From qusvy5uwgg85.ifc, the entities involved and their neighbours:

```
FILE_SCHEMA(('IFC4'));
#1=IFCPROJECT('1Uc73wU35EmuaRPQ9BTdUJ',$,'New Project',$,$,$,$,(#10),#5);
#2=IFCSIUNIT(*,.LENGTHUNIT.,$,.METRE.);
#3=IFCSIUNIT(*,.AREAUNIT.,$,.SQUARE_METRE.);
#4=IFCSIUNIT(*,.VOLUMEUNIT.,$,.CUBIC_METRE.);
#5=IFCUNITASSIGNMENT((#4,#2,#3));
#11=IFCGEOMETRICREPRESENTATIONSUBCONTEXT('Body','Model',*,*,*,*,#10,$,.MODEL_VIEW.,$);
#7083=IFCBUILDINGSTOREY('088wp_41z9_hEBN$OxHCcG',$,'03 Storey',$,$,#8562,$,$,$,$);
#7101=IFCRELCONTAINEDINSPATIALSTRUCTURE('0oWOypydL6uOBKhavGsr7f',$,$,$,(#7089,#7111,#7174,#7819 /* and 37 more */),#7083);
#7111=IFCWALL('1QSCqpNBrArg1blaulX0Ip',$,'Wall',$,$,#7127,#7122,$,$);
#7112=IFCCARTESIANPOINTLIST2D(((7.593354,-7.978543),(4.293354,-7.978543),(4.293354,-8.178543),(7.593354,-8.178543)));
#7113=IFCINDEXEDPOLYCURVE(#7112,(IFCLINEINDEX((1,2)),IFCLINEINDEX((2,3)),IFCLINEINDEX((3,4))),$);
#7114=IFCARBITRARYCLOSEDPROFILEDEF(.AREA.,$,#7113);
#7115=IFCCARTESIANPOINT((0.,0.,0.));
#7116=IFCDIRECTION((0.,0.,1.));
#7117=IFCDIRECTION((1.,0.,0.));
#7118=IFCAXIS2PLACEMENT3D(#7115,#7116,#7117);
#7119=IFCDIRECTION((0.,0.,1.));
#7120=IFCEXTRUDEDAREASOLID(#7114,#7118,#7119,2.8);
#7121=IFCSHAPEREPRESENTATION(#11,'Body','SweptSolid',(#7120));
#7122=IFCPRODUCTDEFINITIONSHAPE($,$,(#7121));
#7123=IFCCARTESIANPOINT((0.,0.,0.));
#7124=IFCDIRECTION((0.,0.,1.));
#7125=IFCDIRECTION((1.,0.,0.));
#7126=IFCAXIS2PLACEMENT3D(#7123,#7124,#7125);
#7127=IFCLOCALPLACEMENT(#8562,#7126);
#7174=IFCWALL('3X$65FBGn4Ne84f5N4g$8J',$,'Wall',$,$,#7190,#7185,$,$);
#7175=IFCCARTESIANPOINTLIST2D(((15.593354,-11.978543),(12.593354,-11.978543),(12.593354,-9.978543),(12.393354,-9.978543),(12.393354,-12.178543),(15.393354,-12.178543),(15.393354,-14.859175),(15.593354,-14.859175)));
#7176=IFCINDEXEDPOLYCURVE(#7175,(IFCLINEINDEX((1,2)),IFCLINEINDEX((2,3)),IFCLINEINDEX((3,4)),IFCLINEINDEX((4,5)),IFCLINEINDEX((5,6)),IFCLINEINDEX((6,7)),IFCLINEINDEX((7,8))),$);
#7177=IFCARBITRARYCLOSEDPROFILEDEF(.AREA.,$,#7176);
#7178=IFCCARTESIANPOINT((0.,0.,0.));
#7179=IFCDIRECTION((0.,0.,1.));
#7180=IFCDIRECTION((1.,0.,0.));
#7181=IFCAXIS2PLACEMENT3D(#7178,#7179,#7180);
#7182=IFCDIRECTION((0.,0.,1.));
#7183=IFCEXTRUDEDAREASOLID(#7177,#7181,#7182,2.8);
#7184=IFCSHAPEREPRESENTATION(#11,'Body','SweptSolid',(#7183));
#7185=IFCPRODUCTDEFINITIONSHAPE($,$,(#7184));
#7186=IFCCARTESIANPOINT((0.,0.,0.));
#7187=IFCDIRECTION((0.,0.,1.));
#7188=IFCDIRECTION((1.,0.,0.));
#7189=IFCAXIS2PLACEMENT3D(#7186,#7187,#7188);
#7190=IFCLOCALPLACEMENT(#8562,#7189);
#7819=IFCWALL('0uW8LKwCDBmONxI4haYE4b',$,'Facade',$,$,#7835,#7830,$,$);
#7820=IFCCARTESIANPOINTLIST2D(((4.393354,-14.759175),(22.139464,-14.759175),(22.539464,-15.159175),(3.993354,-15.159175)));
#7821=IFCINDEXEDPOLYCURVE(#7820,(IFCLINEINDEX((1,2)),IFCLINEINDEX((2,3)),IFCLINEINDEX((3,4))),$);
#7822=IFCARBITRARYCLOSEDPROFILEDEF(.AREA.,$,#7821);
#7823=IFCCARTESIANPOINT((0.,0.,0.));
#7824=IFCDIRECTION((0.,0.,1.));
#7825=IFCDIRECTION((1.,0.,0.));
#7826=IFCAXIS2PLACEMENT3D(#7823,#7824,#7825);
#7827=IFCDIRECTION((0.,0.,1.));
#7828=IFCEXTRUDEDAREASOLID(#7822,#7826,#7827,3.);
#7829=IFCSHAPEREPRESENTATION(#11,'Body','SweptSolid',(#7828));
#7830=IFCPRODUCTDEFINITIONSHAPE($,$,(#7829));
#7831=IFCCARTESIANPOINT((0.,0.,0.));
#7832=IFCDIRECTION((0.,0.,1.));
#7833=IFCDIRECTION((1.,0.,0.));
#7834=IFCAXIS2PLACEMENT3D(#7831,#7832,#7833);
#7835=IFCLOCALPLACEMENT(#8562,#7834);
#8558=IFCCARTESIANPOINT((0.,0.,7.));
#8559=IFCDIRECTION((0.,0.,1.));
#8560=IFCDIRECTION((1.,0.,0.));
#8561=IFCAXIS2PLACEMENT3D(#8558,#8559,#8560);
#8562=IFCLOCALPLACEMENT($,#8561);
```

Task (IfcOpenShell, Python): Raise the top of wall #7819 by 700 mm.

```python
import ifcopenshell
import ifcopenshell.geom
import ifcopenshell.util.representation
import ifcopenshell.util.shape
import ifcopenshell.util.unit

model = ifcopenshell.open("qusvy5uwgg85.ifc")
unit_scale = ifcopenshell.util.unit.calculate_unit_scale(model)
settings = ifcopenshell.geom.settings()


def volume(element):
    """Net volume in cubic metres, openings subtracted."""
    shape = ifcopenshell.geom.create_shape(settings, element)
    return ifcopenshell.util.shape.get_volume(shape.geometry)


wall = model.by_guid("0uW8LKwCDBmONxI4haYE4b")
before = volume(wall)

body = ifcopenshell.util.representation.get_representation(wall, "Model", "Body")
solid = body.Items[0]
old_height = solid.Depth
solid.Depth += 0.7 / unit_scale
after = volume(wall)

print(f"height {old_height:g} -> {solid.Depth:g}, volume {before:.3f} -> {after:.3f} m3")

model.write("qusvy5uwgg85_rev.ifc")
```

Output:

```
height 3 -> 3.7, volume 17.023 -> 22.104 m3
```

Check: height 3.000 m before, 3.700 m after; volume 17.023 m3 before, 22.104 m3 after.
